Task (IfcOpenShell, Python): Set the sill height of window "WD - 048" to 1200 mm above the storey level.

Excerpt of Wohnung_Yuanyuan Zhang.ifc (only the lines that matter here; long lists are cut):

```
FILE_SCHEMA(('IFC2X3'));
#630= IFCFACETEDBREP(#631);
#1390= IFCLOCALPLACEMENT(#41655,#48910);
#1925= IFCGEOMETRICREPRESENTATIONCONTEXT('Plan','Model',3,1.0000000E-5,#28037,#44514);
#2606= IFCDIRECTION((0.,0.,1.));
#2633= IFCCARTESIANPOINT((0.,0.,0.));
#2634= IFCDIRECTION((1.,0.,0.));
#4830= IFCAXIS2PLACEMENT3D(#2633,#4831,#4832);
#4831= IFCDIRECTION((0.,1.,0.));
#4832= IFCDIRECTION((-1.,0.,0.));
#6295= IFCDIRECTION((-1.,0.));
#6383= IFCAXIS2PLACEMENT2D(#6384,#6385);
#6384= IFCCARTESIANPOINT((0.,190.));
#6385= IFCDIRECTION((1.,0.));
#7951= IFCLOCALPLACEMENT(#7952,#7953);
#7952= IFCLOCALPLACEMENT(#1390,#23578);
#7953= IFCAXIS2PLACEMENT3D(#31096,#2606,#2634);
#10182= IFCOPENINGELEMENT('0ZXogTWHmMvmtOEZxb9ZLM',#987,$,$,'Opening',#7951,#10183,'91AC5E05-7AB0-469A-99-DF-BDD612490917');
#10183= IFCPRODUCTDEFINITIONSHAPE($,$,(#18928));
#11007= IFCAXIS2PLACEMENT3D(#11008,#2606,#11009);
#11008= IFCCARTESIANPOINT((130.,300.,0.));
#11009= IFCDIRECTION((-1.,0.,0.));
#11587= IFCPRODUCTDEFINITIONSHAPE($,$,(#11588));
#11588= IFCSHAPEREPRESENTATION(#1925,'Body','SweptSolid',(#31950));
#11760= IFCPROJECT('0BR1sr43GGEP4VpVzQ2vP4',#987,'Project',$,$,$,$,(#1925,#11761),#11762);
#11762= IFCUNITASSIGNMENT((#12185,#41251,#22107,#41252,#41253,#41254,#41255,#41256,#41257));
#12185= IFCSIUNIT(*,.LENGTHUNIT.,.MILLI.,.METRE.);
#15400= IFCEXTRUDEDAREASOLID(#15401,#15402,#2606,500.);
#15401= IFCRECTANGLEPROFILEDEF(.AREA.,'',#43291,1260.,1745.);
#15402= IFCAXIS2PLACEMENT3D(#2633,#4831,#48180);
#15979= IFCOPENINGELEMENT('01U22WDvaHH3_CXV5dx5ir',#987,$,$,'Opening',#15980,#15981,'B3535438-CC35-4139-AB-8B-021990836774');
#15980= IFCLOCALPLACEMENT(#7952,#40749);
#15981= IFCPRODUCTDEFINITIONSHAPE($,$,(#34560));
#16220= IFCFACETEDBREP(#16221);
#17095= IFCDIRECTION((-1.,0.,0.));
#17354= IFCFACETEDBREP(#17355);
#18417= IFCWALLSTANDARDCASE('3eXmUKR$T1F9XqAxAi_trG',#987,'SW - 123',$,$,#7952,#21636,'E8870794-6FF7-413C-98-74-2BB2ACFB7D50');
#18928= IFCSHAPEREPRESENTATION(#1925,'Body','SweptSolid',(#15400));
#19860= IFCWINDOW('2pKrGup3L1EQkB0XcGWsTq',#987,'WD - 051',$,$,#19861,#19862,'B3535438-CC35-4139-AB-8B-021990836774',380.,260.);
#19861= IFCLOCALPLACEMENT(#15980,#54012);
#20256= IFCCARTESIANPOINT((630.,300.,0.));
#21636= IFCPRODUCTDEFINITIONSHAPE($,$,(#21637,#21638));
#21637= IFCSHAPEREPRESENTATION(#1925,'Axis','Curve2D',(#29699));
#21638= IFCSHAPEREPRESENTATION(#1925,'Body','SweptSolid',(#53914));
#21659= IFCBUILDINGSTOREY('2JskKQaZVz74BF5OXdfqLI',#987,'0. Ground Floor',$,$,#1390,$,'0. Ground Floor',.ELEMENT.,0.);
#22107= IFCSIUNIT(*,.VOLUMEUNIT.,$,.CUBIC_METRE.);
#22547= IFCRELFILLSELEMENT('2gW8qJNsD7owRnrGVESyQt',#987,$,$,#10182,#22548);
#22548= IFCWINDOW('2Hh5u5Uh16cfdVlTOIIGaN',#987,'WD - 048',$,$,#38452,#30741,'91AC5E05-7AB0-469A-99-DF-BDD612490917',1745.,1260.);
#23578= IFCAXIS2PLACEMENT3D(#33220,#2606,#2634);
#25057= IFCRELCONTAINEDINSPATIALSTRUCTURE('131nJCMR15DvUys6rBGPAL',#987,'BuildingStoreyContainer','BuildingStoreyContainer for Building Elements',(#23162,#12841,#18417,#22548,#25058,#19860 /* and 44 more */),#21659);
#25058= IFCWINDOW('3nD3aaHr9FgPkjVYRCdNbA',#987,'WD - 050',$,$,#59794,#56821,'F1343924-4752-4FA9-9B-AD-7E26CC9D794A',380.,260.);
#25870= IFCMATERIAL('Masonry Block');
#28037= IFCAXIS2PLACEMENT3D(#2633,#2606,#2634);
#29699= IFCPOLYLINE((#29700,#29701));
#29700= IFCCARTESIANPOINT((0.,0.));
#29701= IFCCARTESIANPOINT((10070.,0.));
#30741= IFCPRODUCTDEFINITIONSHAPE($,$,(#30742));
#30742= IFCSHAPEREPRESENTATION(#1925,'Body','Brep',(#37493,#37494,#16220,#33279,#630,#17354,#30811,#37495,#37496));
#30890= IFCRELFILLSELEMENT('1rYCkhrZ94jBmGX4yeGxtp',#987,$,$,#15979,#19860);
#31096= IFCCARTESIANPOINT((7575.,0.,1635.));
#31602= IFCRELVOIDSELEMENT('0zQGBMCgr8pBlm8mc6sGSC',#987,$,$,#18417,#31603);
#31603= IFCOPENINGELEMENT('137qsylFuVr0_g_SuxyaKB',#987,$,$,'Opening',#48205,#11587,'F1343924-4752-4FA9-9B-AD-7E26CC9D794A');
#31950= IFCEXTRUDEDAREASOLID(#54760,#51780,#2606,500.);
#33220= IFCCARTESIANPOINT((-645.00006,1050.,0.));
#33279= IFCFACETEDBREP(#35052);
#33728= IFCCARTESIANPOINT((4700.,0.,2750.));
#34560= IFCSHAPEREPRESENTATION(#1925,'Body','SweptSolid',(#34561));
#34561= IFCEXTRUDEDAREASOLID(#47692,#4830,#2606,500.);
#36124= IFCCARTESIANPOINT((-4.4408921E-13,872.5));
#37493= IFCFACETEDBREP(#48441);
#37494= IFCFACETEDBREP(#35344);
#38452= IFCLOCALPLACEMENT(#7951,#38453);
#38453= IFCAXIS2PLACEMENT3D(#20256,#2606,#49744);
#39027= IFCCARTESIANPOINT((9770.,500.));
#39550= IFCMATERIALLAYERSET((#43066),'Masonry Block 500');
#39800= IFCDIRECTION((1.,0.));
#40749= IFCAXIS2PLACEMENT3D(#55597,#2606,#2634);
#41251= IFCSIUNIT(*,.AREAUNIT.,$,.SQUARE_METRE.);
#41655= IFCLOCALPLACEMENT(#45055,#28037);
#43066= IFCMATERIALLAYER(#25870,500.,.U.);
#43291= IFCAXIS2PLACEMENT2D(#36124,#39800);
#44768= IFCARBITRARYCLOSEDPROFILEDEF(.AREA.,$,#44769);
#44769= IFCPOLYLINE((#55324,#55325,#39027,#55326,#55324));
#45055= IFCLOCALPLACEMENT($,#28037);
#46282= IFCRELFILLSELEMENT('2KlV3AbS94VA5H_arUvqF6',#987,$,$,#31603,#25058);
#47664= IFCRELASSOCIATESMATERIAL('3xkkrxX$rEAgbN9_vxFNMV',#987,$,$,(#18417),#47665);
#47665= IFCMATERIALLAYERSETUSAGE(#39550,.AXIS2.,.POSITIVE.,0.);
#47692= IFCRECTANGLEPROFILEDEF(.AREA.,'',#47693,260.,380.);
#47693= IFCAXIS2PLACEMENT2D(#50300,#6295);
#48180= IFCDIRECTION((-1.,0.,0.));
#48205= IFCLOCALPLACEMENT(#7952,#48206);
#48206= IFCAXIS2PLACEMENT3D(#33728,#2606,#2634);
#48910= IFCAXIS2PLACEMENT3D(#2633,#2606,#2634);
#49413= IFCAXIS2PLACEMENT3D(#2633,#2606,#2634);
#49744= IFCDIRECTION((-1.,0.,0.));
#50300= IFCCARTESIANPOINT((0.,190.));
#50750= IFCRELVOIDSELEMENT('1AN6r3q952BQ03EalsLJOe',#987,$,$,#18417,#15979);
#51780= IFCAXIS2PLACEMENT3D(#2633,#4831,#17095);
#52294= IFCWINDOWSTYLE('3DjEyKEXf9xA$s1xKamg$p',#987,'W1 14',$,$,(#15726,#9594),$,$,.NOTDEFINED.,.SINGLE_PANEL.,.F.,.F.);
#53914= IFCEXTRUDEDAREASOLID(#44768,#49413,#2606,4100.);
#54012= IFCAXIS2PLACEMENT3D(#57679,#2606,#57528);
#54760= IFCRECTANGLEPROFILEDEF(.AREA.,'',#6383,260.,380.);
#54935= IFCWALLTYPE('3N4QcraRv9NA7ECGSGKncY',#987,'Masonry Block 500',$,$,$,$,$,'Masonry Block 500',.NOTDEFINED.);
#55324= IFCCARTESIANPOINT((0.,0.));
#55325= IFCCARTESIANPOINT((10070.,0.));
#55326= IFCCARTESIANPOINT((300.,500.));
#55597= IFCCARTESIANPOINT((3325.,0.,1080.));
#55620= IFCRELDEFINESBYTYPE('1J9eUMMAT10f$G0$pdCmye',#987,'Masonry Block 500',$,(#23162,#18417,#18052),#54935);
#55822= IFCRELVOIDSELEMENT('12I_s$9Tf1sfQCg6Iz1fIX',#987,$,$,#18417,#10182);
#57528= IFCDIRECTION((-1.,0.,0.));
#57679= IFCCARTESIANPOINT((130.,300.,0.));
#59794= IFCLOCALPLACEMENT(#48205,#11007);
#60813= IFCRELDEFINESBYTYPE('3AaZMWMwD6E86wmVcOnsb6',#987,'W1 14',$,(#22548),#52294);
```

```python
import numpy as np
import ifcopenshell
import ifcopenshell.api.geometry
import ifcopenshell.geom
import ifcopenshell.util.element
import ifcopenshell.util.placement
import ifcopenshell.util.shape
import ifcopenshell.util.unit

model = ifcopenshell.open("Wohnung_Yuanyuan Zhang.ifc")
unit_scale = ifcopenshell.util.unit.calculate_unit_scale(model)

window = model.by_guid("2Hh5u5Uh16cfdVlTOIIGaN")
opening = window.FillsVoids[0].RelatingOpeningElement
storey = ifcopenshell.util.element.get_container(window, ifc_class="IfcBuildingStorey")
level = ifcopenshell.util.placement.get_local_placement(storey.ObjectPlacement)[2, 3]

# The opening's origin need not be at the sill, so measure its lowest point.
shape = ifcopenshell.geom.create_shape(ifcopenshell.geom.settings(), opening)
bottom = ifcopenshell.util.shape.get_shape_bottom_elevation(shape, shape.geometry) / unit_scale
dz = level + 1200.0 - bottom

shift = np.array([0.0, 0.0, dz])
# The window is placed relative to its opening, so it follows when the opening moves.
matrix = ifcopenshell.util.placement.get_local_placement(opening.ObjectPlacement)
matrix[:3, 3] += shift
ifcopenshell.api.geometry.edit_object_placement(
    model, product=opening, matrix=matrix, is_si=False, should_transform_children=True
)

print(f"moved by {dz * unit_scale:+.3f} m")

model.write("Wohnung_Yuanyuan Zhang_edited.ifc")
```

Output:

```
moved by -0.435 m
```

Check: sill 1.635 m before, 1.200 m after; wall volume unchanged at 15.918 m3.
